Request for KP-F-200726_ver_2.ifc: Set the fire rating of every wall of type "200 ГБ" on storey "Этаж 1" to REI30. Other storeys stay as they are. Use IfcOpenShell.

First a look at what the model holds.

```python
import ifcopenshell
import ifcopenshell.util.element

model = ifcopenshell.open("KP-F-200726_ver_2.ifc")
print(model.schema)
storey = next(s for s in model.by_type("IfcBuildingStorey") if s.Name == "Этаж 1")
walls = [e for e in ifcopenshell.util.element.get_decomposition(storey) if e.is_a("IfcWall")]
seen = {}
for e in walls:
    element_type = ifcopenshell.util.element.get_type(e)
    key = (element_type.Name if element_type != e and element_type else None, ifcopenshell.util.element.get_pset(e, "Pset_WallCommon", "FireRating"))
    seen[key] = seen.get(key, 0) + 1
for (name, value), count in sorted(seen.items(), key=str):
    print(count, "x", name, "|", value)
```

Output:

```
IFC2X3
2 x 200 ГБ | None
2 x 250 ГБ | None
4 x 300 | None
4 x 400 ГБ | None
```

```python
import ifcopenshell
import ifcopenshell.api.pset
import ifcopenshell.util.element

model = ifcopenshell.open("KP-F-200726_ver_2.ifc")

storey = next(s for s in model.by_type("IfcBuildingStorey") if s.Name == "Этаж 1")
walls = [e for e in ifcopenshell.util.element.get_decomposition(storey) if e.is_a("IfcWall")]

count = 0
for e in walls:
    element_type = ifcopenshell.util.element.get_type(e)
    if element_type in (None, e) or element_type.Name != "200 ГБ":
        continue
    # add_pset returns the element's existing set when there is one.
    pset = ifcopenshell.api.pset.add_pset(model, product=e, name="Pset_WallCommon")
    ifcopenshell.api.pset.edit_pset(model, pset=pset, properties={"FireRating": "REI30"})
    count += 1

print(count, "walls updated")

model.write("KP-F-200726_ver_2_v2.ifc")
```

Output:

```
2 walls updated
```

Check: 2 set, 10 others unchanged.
